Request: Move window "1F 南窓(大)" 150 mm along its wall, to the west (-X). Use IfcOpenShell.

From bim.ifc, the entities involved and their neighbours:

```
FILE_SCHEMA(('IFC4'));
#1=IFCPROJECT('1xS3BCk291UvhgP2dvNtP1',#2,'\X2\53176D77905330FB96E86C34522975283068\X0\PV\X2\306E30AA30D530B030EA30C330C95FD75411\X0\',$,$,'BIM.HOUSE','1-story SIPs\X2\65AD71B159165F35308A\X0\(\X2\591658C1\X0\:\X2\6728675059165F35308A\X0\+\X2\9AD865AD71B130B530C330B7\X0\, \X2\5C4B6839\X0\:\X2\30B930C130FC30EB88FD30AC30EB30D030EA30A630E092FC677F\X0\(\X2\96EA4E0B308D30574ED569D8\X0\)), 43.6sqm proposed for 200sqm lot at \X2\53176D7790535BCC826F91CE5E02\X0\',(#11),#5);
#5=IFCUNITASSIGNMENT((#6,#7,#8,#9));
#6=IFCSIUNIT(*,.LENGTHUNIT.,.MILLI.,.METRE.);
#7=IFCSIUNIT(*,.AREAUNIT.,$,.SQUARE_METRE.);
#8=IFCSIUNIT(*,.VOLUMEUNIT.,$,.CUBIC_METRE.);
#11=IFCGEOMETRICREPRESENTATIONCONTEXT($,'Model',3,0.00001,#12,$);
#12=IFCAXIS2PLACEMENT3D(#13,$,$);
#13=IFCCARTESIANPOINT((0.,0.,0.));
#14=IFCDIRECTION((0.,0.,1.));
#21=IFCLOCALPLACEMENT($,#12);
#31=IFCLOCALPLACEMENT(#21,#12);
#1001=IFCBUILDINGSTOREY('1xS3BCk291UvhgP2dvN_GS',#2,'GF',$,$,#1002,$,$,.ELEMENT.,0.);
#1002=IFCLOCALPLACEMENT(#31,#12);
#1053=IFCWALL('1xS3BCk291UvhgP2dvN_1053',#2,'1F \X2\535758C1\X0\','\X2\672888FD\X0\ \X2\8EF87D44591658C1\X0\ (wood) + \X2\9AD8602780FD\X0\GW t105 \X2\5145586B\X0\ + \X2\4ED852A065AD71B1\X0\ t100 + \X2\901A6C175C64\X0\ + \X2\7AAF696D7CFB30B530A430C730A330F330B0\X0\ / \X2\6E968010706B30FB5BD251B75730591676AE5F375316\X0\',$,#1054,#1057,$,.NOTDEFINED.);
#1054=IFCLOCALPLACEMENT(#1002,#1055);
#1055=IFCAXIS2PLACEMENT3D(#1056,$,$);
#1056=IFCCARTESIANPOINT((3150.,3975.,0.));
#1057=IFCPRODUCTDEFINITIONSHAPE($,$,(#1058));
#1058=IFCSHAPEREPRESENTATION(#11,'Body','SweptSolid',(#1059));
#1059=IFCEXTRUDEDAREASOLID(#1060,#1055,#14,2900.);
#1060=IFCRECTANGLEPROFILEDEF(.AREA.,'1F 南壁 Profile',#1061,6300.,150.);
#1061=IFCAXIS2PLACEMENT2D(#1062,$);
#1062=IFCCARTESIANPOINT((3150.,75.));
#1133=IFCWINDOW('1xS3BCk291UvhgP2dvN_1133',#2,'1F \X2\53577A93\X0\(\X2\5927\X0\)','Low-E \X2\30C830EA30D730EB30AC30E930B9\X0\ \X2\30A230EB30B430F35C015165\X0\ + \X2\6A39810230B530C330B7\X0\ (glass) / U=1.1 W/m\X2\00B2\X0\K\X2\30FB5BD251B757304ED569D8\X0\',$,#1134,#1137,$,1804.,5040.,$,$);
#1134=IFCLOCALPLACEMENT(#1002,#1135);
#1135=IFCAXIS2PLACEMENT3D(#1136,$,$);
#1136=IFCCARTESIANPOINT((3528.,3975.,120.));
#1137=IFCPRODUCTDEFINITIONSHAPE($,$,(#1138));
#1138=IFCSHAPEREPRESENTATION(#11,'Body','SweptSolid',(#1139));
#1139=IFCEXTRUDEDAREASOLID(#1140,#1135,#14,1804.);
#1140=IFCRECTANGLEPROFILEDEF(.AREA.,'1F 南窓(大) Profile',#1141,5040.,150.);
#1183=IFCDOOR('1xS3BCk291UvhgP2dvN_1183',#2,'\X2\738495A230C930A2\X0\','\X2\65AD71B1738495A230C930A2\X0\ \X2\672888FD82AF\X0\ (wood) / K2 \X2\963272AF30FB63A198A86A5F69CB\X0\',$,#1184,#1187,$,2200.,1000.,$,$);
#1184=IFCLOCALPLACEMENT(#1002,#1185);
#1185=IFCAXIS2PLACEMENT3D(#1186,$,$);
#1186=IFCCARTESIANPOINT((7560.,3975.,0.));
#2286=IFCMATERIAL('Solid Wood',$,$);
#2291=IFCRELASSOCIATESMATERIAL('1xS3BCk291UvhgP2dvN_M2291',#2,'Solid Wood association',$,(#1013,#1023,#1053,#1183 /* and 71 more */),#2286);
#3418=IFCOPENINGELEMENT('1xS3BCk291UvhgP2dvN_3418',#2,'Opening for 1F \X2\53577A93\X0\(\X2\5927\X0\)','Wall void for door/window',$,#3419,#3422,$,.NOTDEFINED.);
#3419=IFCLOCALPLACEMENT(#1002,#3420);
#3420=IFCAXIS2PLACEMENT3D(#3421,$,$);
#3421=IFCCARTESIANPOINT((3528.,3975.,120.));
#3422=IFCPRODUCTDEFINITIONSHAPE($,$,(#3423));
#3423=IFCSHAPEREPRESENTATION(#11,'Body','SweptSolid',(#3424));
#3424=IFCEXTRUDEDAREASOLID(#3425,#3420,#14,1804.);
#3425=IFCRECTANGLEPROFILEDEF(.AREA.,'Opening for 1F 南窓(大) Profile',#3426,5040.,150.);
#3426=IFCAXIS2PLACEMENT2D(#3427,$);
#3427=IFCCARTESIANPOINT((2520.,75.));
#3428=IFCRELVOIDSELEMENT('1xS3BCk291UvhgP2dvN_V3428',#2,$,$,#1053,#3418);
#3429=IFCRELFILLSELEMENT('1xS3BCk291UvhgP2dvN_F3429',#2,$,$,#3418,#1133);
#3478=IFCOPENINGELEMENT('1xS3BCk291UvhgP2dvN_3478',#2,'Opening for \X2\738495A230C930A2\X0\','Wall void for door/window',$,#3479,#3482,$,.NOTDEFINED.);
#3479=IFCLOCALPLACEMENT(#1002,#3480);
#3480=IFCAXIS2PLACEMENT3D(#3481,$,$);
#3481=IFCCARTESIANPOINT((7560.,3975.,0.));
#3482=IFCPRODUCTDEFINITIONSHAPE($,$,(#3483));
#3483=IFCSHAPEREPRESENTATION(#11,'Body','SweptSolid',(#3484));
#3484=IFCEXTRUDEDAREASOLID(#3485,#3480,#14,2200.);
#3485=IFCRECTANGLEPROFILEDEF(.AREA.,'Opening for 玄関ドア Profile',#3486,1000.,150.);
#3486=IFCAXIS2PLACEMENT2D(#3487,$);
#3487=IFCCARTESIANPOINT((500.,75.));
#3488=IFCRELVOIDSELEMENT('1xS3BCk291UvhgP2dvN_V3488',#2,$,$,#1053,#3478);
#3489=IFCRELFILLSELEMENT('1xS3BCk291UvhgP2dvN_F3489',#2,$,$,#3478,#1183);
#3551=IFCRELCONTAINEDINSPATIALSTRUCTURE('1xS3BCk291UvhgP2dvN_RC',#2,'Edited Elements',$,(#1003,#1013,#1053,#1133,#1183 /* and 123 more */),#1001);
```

```python
import ifcopenshell
import ifcopenshell.api.geometry
import ifcopenshell.util.placement

model = ifcopenshell.open("bim.ifc")

window = model.by_guid("1xS3BCk291UvhgP2dvN_1133")
opening = window.FillsVoids[0].RelatingOpeningElement
wall = opening.VoidsElements[0].RelatingBuildingElement

wall_matrix = ifcopenshell.util.placement.get_local_placement(wall.ObjectPlacement)
shift = wall_matrix[:3, 0] * -150.0
before = ifcopenshell.util.placement.get_local_placement(window.ObjectPlacement)[:3, 3].copy()

# The window is not placed relative to its opening, so move both.
for product in (opening, window):
    matrix = ifcopenshell.util.placement.get_local_placement(product.ObjectPlacement)
    matrix[:3, 3] += shift
    ifcopenshell.api.geometry.edit_object_placement(model, product=product, matrix=matrix, is_si=False)

after = ifcopenshell.util.placement.get_local_placement(window.ObjectPlacement)[:3, 3]
print("window moved by", (after - before).round(3) + 0.0)

model.write("bim_edited.ifc")
```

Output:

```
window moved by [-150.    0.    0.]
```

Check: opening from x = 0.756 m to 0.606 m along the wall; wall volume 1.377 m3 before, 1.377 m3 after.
